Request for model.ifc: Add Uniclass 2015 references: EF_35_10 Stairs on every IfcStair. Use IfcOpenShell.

First a look at what the model holds.

```python
import ifcopenshell

model = ifcopenshell.open("model.ifc")
print(model.schema)
print("classifications:", [c.Name for c in model.by_type("IfcClassification")])
for ifc_class in ("IfcDoor", "IfcRoof", "IfcStair", "IfcWall", "IfcWindow"):
    print(ifc_class, len(model.by_type(ifc_class)))
```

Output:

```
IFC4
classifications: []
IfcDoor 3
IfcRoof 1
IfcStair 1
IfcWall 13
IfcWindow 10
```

```python
import ifcopenshell
import ifcopenshell.api.classification

model = ifcopenshell.open("model.ifc")

system = ifcopenshell.api.classification.add_classification(model, classification="Uniclass 2015")

codes = {
    "IfcStair": ("EF_35_10", "Stairs"),
}
for ifc_class, (code, name) in codes.items():
    products = model.by_type(ifc_class)
    ifcopenshell.api.classification.add_reference(
        model, products=products, classification=system, identification=code, name=name
    )
    print(code, len(products))

model.write("model_updated.ifc")
```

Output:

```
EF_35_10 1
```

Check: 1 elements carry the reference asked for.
